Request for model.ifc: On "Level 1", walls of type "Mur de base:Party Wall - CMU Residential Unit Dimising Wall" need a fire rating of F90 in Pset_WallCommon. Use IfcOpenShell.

First a look at what the model holds.

```python
import ifcopenshell
import ifcopenshell.util.element

model = ifcopenshell.open("model.ifc")
print(model.schema)
storey = next(s for s in model.by_type("IfcBuildingStorey") if s.Name == "Level 1")
walls = [e for e in ifcopenshell.util.element.get_decomposition(storey) if e.is_a("IfcWall")]
seen = {}
for e in walls:
    element_type = ifcopenshell.util.element.get_type(e)
    key = (element_type.Name if element_type != e and element_type else None, ifcopenshell.util.element.get_pset(e, "Pset_WallCommon", "FireRating"))
    seen[key] = seen.get(key, 0) + 1
for (name, value), count in sorted(seen.items(), key=str):
    print(count, "x", name, "|", value)
```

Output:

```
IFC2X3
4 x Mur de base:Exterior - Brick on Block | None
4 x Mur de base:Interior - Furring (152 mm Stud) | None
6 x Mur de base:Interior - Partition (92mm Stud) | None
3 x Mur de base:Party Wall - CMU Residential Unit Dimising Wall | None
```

```python
import ifcopenshell
import ifcopenshell.api.pset
import ifcopenshell.util.element

model = ifcopenshell.open("model.ifc")

storey = next(s for s in model.by_type("IfcBuildingStorey") if s.Name == "Level 1")
walls = [e for e in ifcopenshell.util.element.get_decomposition(storey) if e.is_a("IfcWall")]

count = 0
for e in walls:
    element_type = ifcopenshell.util.element.get_type(e)
    if element_type in (None, e) or element_type.Name != "Mur de base:Party Wall - CMU Residential Unit Dimising Wall":
        continue
    # add_pset returns the element's existing set when there is one.
    pset = ifcopenshell.api.pset.add_pset(model, product=e, name="Pset_WallCommon")
    ifcopenshell.api.pset.edit_pset(model, pset=pset, properties={"FireRating": "F90"})
    count += 1

print(count, "walls updated")

model.write("model_rev.ifc")
```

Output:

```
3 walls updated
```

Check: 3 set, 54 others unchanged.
